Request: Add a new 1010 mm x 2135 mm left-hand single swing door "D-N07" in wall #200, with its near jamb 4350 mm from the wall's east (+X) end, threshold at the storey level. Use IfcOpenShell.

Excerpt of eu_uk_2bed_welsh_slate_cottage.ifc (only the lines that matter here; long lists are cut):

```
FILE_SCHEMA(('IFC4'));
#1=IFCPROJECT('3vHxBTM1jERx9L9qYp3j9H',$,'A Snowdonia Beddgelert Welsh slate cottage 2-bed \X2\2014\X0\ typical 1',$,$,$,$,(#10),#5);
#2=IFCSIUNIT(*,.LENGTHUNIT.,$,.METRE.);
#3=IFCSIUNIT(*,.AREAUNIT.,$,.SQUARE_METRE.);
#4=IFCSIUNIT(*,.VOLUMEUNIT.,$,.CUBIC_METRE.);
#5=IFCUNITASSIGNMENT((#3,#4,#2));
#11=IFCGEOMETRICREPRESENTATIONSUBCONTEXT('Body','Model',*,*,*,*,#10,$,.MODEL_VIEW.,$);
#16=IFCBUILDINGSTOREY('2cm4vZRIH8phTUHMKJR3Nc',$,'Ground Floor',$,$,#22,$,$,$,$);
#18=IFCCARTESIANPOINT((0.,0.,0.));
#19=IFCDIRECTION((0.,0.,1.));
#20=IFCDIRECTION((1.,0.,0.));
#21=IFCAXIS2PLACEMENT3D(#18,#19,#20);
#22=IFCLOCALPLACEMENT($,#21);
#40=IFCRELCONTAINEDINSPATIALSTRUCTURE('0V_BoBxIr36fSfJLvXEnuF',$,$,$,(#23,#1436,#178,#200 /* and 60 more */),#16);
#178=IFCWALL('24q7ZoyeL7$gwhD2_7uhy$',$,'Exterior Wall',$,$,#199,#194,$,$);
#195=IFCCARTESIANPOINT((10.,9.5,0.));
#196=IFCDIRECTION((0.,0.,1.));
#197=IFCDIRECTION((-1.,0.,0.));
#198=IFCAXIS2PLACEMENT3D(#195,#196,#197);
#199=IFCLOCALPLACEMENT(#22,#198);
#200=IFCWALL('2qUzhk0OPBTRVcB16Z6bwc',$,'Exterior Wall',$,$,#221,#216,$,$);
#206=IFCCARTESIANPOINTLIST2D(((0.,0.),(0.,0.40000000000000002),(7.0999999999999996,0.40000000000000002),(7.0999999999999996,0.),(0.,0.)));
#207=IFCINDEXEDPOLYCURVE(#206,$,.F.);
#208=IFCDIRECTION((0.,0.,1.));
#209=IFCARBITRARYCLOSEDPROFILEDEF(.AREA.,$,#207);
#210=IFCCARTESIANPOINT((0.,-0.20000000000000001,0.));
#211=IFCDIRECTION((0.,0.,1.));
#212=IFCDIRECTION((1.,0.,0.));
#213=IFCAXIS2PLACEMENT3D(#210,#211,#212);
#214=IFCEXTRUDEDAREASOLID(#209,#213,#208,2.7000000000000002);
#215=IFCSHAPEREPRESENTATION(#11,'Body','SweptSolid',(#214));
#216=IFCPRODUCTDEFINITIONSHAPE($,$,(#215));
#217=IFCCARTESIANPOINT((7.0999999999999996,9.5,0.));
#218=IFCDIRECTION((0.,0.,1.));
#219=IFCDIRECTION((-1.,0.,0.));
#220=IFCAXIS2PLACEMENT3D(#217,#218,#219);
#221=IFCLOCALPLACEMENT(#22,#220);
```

```python
import numpy as np
import ifcopenshell
import ifcopenshell.api.feature
import ifcopenshell.api.geometry
import ifcopenshell.api.root
import ifcopenshell.api.spatial
import ifcopenshell.geom
import ifcopenshell.util.element
import ifcopenshell.util.placement
import ifcopenshell.util.representation
import ifcopenshell.util.shape
import ifcopenshell.util.unit

model = ifcopenshell.open("eu_uk_2bed_welsh_slate_cottage.ifc")
unit_scale = ifcopenshell.util.unit.calculate_unit_scale(model)
settings = ifcopenshell.geom.settings()


def volume(element):
    """Net volume in cubic metres, openings subtracted."""
    shape = ifcopenshell.geom.create_shape(settings, element)
    return ifcopenshell.util.shape.get_volume(shape.geometry)


wall = model.by_id(200)
storey = ifcopenshell.util.element.get_container(wall, ifc_class="IfcBuildingStorey")
context = ifcopenshell.util.representation.get_context(model, "Model", "Body", "MODEL_VIEW")
before = volume(wall)

width, height, from_end, sill = 1.01, 2.135, 4.35, 0.0  # metres

# The wall runs along its own X axis, and the end named is its -X end.
wall_shape = ifcopenshell.geom.create_shape(settings, wall)
x, y, z = ifcopenshell.util.shape.get_vertices(wall_shape.geometry).T
start = x.min() + from_end
face, thickness = float(y.min()), float(y.max() - y.min())
wall_matrix = ifcopenshell.util.placement.get_local_placement(wall.ObjectPlacement)
level = ifcopenshell.util.placement.get_local_placement(storey.ObjectPlacement)[2, 3]


def in_wall(x, y):
    """Placement at x, y metres in the wall's axes, at sill height."""
    matrix = wall_matrix.copy()
    matrix[:, 3] = wall_matrix @ np.array([x / unit_scale, y / unit_scale, 0.0, 1.0])
    matrix[2, 3] = level + sill / unit_scale
    return matrix


# Opening: a box that overshoots both wall faces by 50 mm.
opening = ifcopenshell.api.root.create_entity(model, ifc_class="IfcOpeningElement", predefined_type="OPENING")
box = ifcopenshell.api.geometry.add_wall_representation(
    model, context=context, length=width, height=height, thickness=thickness + 0.1
)
ifcopenshell.api.geometry.assign_representation(model, product=opening, representation=box)
ifcopenshell.api.geometry.edit_object_placement(model, product=opening, matrix=in_wall(start, face - 0.05), is_si=False)
ifcopenshell.api.feature.add_feature(model, feature=opening, element=wall)

door = ifcopenshell.api.root.create_entity(model, ifc_class="IfcDoor", name="D-N07", predefined_type="DOOR")
door.OverallWidth, door.OverallHeight = width / unit_scale, height / unit_scale
door.OperationType = "SINGLE_SWING_LEFT"
body = ifcopenshell.api.geometry.add_door_representation(
    model,
    context=context,
    overall_width=door.OverallWidth,
    overall_height=door.OverallHeight,
    operation_type="SINGLE_SWING_LEFT",
    lining_properties={"LiningDepth": thickness / unit_scale, "ThresholdDepth": thickness / unit_scale},
)
ifcopenshell.api.geometry.assign_representation(model, product=door, representation=body)
ifcopenshell.api.spatial.assign_container(model, products=[door], relating_structure=storey)
ifcopenshell.api.feature.add_filling(model, opening=opening, element=door)

# The lining spans the wall, so the door starts at the wall face.
ifcopenshell.api.geometry.edit_object_placement(model, product=door, matrix=in_wall(start, face), is_si=False)

after = volume(wall)

print(f"wall volume {before:.3f} -> {after:.3f} m3")

model.write("eu_uk_2bed_welsh_slate_cottage_updated.ifc")
```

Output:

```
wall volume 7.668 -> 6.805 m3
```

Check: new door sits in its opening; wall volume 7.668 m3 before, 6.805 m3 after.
